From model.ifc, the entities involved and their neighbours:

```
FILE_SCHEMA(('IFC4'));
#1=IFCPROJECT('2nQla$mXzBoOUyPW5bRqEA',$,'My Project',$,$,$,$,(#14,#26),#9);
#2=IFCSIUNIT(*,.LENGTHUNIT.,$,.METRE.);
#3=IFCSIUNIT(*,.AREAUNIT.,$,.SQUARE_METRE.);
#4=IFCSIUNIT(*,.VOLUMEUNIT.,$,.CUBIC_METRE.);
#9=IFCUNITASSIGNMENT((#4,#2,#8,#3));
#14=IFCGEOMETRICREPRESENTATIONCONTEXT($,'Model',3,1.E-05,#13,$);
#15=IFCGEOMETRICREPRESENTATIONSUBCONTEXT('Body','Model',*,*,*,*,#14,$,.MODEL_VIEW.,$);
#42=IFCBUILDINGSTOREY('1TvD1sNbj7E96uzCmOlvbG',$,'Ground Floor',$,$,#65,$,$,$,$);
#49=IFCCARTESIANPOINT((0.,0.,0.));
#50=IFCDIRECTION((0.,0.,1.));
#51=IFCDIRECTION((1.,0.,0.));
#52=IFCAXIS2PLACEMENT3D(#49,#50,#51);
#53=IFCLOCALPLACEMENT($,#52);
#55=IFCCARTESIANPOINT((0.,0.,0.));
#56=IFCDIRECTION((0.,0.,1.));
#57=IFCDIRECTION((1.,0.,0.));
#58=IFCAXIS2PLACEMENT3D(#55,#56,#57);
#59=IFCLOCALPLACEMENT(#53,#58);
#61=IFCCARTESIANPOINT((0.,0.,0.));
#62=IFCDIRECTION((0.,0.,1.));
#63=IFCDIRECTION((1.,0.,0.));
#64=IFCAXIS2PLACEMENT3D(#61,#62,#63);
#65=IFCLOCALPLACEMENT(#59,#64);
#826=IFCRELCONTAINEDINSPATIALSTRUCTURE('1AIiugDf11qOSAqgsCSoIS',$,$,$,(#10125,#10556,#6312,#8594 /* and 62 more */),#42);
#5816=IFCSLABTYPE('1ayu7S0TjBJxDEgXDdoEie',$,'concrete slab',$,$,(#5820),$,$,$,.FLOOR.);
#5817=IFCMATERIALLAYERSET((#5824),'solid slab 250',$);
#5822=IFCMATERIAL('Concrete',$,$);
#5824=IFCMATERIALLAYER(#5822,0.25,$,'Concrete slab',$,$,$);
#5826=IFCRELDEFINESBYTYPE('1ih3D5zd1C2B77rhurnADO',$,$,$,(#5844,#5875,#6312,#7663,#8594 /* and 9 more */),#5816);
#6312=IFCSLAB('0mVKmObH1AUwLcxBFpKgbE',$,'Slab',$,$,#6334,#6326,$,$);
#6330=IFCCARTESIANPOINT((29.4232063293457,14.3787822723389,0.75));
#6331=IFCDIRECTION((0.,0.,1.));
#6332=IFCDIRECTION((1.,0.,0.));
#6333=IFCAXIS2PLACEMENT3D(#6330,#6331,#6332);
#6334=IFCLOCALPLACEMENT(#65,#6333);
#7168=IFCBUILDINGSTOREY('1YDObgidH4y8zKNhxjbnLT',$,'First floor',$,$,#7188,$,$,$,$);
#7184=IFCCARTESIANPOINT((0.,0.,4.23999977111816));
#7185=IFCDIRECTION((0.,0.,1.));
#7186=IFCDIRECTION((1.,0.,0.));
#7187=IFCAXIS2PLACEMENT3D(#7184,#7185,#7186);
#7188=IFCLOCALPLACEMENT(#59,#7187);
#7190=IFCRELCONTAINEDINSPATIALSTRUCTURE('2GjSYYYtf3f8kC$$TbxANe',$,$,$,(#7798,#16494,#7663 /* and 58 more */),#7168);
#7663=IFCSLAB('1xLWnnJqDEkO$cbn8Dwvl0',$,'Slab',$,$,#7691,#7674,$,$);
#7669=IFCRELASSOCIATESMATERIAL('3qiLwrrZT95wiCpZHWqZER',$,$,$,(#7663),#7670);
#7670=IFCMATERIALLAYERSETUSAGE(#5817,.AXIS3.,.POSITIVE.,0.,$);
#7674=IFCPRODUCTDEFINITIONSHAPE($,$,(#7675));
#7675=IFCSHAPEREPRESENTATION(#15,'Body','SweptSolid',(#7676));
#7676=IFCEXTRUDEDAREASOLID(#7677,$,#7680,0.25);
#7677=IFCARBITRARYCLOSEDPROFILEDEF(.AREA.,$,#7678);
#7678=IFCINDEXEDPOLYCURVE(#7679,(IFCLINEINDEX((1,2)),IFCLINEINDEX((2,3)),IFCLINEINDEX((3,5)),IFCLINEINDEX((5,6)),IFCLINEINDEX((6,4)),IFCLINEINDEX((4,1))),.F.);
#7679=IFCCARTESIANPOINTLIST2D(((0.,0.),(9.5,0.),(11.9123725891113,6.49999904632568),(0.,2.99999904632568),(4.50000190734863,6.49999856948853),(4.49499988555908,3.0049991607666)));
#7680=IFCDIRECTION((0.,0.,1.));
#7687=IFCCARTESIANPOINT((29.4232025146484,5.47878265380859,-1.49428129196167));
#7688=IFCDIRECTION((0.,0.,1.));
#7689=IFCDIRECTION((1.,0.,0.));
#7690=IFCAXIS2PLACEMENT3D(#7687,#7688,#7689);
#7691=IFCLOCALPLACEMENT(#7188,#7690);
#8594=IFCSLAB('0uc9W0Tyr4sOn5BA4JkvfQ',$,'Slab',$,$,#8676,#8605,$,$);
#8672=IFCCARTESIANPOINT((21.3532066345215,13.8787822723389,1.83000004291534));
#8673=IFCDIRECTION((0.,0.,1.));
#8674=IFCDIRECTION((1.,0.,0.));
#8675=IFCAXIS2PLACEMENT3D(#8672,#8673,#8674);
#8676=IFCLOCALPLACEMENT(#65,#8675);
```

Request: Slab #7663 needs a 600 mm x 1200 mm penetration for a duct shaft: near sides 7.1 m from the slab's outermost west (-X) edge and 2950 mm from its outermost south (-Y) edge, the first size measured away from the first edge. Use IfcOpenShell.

```python
import numpy as np
import ifcopenshell
import ifcopenshell.api.feature
import ifcopenshell.api.geometry
import ifcopenshell.api.root
import ifcopenshell.geom
import ifcopenshell.util.placement
import ifcopenshell.util.representation
import ifcopenshell.util.shape
import ifcopenshell.util.unit

model = ifcopenshell.open("model.ifc")
unit_scale = ifcopenshell.util.unit.calculate_unit_scale(model)
settings = ifcopenshell.geom.settings()


def volume(element):
    """Net volume in cubic metres, openings subtracted."""
    shape = ifcopenshell.geom.create_shape(settings, element)
    return ifcopenshell.util.shape.get_volume(shape.geometry)


slab = model.by_guid("1xLWnnJqDEkO$cbn8Dwvl0")
before = volume(slab)

# Extent in the slab's own axes, in metres. The edges named are its -X and -Y sides.
slab_shape = ifcopenshell.geom.create_shape(settings, slab)
vertices = ifcopenshell.util.shape.get_vertices(slab_shape.geometry)
x_min, y_min, bottom = vertices.min(axis=0)
top = vertices[:, 2].max()

opening = ifcopenshell.api.root.create_entity(model, ifc_class="IfcOpeningElement", name="Duct shaft opening", predefined_type="OPENING")
context = ifcopenshell.util.representation.get_context(model, "Model", "Body", "MODEL_VIEW")
width, depth = 0.6, 1.2
outline = [(0.0, 0.0), (width, 0.0), (width, depth), (0.0, depth), (0.0, 0.0)]
# Overshoot both faces by 50 mm so the cut is clean.
shape = ifcopenshell.api.geometry.add_slab_representation(
    model, context=context, depth=top - bottom + 0.1, polyline=outline
)
ifcopenshell.api.geometry.assign_representation(model, product=opening, representation=shape)

matrix = ifcopenshell.util.placement.get_local_placement(slab.ObjectPlacement)
matrix[:, 3] = matrix @ np.append(np.array([x_min + 7.1, y_min + 2.95, bottom - 0.05]) / unit_scale, 1.0)
ifcopenshell.api.geometry.edit_object_placement(model, product=opening, matrix=matrix, is_si=False)
ifcopenshell.api.feature.add_feature(model, feature=opening, element=slab)

after = volume(slab)

print(f"slab volume {before:.3f} -> {after:.3f} m3")

model.write("model_v2.ifc")
```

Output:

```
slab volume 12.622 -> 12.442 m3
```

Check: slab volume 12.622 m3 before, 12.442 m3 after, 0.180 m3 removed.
